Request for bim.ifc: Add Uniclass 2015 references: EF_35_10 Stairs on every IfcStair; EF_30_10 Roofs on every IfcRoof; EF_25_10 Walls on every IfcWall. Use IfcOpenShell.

First a look at what the model holds.

```python
import ifcopenshell

model = ifcopenshell.open("bim.ifc")
print(model.schema)
print("classifications:", [c.Name for c in model.by_type("IfcClassification")])
for ifc_class in ("IfcDoor", "IfcRoof", "IfcStair", "IfcWall", "IfcWindow"):
    print(ifc_class, len(model.by_type(ifc_class)))
```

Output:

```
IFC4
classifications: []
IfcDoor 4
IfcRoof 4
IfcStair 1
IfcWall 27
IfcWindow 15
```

```python
import ifcopenshell
import ifcopenshell.api.classification

model = ifcopenshell.open("bim.ifc")

system = ifcopenshell.api.classification.add_classification(model, classification="Uniclass 2015")

codes = {
    "IfcStair": ("EF_35_10", "Stairs"),
    "IfcRoof": ("EF_30_10", "Roofs"),
    "IfcWall": ("EF_25_10", "Walls"),
}
for ifc_class, (code, name) in codes.items():
    products = model.by_type(ifc_class)
    ifcopenshell.api.classification.add_reference(
        model, products=products, classification=system, identification=code, name=name
    )
    print(code, len(products))

model.write("bim_updated.ifc")
```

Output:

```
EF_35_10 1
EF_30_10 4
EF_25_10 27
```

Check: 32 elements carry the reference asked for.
